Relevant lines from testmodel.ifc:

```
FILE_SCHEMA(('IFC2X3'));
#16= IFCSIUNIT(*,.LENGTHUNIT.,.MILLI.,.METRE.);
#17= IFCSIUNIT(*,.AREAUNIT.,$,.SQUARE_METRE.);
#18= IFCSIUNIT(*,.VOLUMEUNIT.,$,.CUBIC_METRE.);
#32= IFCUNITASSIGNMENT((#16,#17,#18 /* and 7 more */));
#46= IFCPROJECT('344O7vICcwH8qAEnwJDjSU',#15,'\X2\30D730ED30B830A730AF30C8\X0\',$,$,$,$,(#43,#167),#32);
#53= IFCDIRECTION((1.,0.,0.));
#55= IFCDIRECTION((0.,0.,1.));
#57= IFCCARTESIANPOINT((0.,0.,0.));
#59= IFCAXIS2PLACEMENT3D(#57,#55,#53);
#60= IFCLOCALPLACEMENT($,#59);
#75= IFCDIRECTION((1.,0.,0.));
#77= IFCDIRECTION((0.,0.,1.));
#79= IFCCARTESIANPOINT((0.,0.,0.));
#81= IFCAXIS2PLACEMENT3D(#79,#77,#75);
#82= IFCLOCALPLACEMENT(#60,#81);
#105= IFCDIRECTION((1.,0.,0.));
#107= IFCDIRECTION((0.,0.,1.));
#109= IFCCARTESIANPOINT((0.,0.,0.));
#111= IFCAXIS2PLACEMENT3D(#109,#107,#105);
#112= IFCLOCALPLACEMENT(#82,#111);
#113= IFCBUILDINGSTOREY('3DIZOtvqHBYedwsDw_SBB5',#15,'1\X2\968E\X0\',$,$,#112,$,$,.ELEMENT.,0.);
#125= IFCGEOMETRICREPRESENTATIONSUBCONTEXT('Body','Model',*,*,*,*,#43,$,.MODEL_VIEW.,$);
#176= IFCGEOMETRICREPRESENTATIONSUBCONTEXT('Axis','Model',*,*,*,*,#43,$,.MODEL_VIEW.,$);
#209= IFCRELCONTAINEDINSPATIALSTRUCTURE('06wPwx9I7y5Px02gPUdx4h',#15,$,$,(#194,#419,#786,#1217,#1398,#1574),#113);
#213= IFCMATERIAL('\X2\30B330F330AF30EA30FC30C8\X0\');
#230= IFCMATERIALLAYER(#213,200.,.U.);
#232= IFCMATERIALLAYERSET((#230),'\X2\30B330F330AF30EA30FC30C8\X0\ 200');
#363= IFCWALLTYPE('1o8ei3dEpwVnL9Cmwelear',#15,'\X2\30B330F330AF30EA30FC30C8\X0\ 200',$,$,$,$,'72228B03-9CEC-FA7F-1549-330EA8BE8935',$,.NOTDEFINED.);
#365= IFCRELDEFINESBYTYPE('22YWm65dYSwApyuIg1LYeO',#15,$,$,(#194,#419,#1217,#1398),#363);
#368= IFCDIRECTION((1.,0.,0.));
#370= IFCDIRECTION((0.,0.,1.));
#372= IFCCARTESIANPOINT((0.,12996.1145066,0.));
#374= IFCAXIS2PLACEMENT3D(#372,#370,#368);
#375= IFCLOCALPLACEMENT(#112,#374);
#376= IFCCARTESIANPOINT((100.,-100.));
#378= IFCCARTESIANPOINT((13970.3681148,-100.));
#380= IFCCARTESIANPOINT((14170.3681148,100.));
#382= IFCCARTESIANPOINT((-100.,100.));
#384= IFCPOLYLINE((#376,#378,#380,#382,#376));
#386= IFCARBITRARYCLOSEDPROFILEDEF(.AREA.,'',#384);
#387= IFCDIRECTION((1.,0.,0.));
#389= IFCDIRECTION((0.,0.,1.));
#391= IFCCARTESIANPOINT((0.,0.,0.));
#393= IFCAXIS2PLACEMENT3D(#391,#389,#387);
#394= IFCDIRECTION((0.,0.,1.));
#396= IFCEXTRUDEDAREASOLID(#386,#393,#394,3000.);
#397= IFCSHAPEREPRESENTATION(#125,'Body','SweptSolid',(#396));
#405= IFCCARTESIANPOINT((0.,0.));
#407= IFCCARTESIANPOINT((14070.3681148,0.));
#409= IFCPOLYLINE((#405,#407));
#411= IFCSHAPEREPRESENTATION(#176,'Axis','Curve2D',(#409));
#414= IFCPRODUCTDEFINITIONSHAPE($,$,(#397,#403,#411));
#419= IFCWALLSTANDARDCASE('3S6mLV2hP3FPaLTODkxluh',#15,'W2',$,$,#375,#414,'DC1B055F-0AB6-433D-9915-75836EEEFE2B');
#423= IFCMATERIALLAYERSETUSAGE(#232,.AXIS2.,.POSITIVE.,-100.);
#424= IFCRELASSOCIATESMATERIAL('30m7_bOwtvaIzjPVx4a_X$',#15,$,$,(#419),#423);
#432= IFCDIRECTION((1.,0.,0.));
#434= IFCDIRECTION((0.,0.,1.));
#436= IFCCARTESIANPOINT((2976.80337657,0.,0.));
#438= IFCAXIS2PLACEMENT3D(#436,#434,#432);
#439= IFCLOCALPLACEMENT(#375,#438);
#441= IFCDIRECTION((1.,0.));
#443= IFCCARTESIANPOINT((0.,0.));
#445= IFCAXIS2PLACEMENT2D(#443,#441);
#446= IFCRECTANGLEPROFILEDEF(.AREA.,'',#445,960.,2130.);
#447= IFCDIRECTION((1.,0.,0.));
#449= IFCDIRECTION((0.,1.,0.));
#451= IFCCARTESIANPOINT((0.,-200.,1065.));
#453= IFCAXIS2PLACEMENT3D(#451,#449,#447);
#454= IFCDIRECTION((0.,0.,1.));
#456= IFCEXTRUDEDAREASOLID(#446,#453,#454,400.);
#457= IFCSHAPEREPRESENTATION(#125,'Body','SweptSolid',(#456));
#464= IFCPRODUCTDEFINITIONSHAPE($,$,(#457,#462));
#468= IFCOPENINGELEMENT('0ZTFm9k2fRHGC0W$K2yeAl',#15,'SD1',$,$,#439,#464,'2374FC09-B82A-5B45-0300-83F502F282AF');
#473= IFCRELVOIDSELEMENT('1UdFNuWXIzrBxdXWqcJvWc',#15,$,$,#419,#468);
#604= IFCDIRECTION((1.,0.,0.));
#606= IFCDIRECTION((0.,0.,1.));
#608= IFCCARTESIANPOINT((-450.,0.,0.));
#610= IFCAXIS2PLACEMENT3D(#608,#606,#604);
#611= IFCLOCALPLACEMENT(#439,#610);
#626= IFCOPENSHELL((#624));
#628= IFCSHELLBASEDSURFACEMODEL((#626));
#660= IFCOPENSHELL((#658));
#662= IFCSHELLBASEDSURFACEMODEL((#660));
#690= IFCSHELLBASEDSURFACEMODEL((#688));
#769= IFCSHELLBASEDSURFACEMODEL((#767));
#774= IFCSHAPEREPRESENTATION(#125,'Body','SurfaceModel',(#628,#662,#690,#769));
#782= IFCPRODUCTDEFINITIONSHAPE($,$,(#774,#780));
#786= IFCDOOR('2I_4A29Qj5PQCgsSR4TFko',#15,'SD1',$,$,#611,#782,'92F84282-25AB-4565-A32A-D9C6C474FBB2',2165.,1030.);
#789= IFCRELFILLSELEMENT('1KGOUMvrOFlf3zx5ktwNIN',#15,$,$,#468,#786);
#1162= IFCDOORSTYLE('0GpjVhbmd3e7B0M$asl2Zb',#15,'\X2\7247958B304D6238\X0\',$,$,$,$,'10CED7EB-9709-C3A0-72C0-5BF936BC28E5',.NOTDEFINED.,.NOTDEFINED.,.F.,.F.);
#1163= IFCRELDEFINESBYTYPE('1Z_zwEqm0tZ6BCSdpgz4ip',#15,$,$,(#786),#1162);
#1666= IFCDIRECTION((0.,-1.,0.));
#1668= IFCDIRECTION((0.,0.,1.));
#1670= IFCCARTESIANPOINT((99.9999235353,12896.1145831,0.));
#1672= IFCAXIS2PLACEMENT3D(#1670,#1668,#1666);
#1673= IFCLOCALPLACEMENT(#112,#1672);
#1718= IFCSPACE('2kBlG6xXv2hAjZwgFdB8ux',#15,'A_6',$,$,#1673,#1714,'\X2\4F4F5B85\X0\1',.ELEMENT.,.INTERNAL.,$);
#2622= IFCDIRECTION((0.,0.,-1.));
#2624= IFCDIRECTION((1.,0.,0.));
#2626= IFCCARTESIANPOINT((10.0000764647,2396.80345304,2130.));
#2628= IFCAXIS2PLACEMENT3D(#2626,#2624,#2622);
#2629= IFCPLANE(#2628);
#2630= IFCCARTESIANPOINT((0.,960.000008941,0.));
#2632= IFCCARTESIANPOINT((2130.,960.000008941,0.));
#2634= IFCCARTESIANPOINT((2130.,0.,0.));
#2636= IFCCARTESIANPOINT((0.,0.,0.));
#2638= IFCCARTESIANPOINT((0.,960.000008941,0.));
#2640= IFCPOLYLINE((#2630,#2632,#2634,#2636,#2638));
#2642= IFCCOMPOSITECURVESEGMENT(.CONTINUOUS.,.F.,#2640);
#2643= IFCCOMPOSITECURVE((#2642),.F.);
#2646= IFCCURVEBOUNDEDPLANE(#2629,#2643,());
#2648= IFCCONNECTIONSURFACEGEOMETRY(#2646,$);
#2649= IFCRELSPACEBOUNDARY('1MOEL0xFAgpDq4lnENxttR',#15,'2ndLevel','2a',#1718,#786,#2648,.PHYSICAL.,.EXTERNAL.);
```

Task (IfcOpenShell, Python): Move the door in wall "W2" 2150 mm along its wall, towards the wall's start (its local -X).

```python
import numpy as np
import ifcopenshell
import ifcopenshell.api.geometry
import ifcopenshell.util.placement
import ifcopenshell.util.unit

model = ifcopenshell.open("testmodel.ifc")
unit_scale = ifcopenshell.util.unit.calculate_unit_scale(model)

door = model.by_id(786)
opening = door.FillsVoids[0].RelatingOpeningElement
wall = opening.VoidsElements[0].RelatingBuildingElement

wall_matrix = ifcopenshell.util.placement.get_local_placement(wall.ObjectPlacement)
shift = wall_matrix[:3, 0] * -2.15 / unit_scale
before = ifcopenshell.util.placement.get_local_placement(door.ObjectPlacement)[:3, 3].copy()

# The door is placed relative to its opening, so it follows when the opening moves.
matrix = ifcopenshell.util.placement.get_local_placement(opening.ObjectPlacement)
matrix[:3, 3] += shift
ifcopenshell.api.geometry.edit_object_placement(
    model, product=opening, matrix=matrix, is_si=False, should_transform_children=True
)

# Space boundary surfaces are stored in each space's coordinates; move them too.
for rel in door.ProvidesBoundaries:
    if not rel.ConnectionGeometry:
        continue
    surface = rel.ConnectionGeometry.SurfaceOnRelatingElement.BasisSurface
    space_matrix = ifcopenshell.util.placement.get_local_placement(rel.RelatingSpace.ObjectPlacement)
    point = np.array(surface.Position.Location.Coordinates) + space_matrix[:3, :3].T @ shift
    surface.Position = model.createIfcAxis2Placement3D(
        model.createIfcCartesianPoint(point.tolist()), surface.Position.Axis, surface.Position.RefDirection
    )

after = ifcopenshell.util.placement.get_local_placement(door.ObjectPlacement)[:3, 3]
print("door moved by", (after - before).round(3) + 0.0)

model.write("testmodel_updated.ifc")
```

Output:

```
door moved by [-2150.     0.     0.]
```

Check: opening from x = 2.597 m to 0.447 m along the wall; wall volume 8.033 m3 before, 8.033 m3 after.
